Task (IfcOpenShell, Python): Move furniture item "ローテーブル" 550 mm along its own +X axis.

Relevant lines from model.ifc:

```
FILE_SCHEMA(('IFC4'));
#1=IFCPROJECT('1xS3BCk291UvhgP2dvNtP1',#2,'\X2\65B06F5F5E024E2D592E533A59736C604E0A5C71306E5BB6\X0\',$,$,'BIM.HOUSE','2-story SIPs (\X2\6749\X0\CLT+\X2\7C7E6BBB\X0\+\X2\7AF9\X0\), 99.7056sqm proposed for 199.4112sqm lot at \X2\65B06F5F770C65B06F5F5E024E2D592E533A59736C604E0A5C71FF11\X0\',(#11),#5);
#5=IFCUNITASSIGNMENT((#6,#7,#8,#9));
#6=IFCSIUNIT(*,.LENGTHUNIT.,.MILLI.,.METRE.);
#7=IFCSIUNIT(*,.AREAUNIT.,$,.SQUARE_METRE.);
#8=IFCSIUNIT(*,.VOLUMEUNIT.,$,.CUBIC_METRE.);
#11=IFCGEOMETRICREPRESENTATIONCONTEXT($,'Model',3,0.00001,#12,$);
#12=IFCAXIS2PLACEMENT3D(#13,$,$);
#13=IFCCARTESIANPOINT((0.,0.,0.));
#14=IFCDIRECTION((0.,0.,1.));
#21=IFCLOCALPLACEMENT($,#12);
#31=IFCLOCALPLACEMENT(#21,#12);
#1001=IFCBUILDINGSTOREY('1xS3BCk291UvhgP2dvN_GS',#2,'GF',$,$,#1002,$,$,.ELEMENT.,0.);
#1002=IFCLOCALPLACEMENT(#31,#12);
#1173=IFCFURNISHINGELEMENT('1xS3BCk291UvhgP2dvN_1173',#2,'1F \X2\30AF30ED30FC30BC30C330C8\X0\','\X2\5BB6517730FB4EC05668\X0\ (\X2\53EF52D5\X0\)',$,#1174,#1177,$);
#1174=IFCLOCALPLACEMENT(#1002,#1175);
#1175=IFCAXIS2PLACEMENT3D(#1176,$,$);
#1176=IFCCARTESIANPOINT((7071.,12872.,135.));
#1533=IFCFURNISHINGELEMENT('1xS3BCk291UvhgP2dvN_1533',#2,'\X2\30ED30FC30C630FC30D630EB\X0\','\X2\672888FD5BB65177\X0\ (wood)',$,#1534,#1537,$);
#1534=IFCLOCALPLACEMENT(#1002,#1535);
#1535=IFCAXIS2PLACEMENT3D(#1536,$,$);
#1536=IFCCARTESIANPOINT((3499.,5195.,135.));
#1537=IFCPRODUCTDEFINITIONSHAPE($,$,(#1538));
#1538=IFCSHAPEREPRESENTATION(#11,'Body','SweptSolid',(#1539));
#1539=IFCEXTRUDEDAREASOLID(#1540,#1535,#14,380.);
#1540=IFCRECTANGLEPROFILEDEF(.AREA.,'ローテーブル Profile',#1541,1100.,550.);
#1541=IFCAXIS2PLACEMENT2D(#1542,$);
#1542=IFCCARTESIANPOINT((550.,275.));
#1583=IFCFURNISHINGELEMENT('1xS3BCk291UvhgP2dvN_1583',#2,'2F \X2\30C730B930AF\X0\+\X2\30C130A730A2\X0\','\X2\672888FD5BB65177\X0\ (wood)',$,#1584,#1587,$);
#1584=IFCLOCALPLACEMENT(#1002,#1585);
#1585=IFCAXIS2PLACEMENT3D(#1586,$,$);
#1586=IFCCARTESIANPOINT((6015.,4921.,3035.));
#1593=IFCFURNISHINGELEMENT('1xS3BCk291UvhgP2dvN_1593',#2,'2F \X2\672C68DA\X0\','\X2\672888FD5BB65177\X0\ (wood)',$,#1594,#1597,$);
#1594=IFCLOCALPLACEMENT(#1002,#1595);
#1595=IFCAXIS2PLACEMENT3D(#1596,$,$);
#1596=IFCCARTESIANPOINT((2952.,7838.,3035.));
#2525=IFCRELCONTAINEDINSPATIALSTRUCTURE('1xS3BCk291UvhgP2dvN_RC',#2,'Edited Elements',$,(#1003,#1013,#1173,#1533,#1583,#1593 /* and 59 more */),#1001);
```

```python
import ifcopenshell
import ifcopenshell.api.geometry
import ifcopenshell.util.placement
import ifcopenshell.util.unit

model = ifcopenshell.open("model.ifc")
unit_scale = ifcopenshell.util.unit.calculate_unit_scale(model)

item = model.by_guid("1xS3BCk291UvhgP2dvN_1533")
matrix = ifcopenshell.util.placement.get_local_placement(item.ObjectPlacement)
matrix[:3, 3] += matrix[:3, 0] * 0.55 / unit_scale
ifcopenshell.api.geometry.edit_object_placement(model, product=item, matrix=matrix, is_si=False)

print(ifcopenshell.util.placement.get_local_placement(item.ObjectPlacement).round(3) + 0.0)

model.write("model-out.ifc")
```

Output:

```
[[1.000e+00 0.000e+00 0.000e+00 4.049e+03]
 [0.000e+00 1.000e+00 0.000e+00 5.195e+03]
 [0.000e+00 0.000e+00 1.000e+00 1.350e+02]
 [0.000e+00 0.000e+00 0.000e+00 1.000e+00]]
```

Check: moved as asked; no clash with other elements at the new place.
